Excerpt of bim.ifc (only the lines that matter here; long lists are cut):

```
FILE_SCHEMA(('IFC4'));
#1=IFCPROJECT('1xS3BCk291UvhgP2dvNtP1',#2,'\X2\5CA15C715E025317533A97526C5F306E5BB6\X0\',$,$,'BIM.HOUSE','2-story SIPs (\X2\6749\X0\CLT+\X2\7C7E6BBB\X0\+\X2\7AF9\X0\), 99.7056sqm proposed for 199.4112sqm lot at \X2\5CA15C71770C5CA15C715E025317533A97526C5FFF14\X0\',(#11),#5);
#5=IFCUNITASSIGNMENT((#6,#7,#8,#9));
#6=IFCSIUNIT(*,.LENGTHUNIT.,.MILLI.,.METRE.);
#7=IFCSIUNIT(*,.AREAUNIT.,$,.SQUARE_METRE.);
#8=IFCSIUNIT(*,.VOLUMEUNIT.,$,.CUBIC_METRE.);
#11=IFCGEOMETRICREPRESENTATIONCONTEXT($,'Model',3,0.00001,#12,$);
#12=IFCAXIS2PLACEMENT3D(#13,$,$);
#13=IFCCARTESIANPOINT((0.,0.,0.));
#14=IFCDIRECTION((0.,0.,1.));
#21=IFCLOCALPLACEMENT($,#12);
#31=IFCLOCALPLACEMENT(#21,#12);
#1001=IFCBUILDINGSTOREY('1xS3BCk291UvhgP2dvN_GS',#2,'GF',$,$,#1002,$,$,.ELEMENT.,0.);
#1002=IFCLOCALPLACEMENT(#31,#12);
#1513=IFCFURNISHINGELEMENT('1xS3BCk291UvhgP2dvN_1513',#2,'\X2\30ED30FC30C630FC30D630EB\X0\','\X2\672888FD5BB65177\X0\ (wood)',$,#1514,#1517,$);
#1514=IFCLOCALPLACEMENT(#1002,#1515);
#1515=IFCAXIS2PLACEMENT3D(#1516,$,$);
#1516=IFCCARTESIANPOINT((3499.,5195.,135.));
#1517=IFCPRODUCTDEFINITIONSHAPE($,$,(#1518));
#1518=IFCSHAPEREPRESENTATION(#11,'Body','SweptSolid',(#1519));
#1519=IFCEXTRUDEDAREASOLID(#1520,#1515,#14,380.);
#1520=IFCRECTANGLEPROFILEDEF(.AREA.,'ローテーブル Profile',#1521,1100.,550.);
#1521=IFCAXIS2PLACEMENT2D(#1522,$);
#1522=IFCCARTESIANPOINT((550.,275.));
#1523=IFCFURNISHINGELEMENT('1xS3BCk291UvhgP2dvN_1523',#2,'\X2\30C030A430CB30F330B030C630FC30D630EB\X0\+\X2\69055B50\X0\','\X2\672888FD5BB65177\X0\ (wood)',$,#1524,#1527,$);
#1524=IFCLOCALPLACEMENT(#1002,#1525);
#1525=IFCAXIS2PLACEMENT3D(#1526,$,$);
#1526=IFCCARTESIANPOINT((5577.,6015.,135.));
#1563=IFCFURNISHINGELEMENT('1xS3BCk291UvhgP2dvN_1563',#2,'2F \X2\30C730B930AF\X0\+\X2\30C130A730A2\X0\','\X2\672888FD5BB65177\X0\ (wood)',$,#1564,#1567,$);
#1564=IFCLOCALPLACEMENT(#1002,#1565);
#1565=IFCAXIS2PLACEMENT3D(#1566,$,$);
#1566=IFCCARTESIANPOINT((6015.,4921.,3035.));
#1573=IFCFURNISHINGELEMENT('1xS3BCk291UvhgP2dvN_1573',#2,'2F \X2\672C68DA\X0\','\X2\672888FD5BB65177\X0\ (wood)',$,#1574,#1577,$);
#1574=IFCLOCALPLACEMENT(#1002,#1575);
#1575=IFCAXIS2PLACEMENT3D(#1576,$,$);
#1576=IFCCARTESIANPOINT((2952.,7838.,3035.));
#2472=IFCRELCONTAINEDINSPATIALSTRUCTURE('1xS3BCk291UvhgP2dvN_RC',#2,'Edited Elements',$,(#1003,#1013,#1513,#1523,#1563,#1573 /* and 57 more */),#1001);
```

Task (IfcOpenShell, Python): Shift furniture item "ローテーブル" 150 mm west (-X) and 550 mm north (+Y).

```python
import ifcopenshell
import ifcopenshell.api.geometry
import ifcopenshell.util.placement

model = ifcopenshell.open("bim.ifc")

item = model.by_guid("1xS3BCk291UvhgP2dvN_1513")
matrix = ifcopenshell.util.placement.get_local_placement(item.ObjectPlacement)
matrix[0, 3] -= 150.0
matrix[1, 3] += 550.0
ifcopenshell.api.geometry.edit_object_placement(model, product=item, matrix=matrix, is_si=False)

print(ifcopenshell.util.placement.get_local_placement(item.ObjectPlacement).round(3) + 0.0)

model.write("bim_edited.ifc")
```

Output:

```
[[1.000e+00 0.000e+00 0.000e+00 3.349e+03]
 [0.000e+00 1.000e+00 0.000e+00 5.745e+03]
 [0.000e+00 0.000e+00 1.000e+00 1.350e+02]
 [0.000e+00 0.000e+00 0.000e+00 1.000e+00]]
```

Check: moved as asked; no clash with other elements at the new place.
